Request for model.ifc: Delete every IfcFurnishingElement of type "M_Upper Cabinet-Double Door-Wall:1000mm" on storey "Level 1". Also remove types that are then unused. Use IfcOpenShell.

First a look at what the model holds.

```python
import ifcopenshell
import ifcopenshell.util.element

model = ifcopenshell.open("model.ifc")
print(model.schema)
storey = next(s for s in model.by_type("IfcBuildingStorey") if s.Name == "Level 1")
furniture = [e for e in ifcopenshell.util.element.get_decomposition(storey) if e.is_a("IfcFurnishingElement")]
seen = {}
for e in furniture:
    element_type = ifcopenshell.util.element.get_type(e)
    name = element_type.Name if element_type not in (None, e) else None
    seen[name] = seen.get(name, 0) + 1
for name, count in sorted(seen.items(), key=str):
    print(count, "x", name)
```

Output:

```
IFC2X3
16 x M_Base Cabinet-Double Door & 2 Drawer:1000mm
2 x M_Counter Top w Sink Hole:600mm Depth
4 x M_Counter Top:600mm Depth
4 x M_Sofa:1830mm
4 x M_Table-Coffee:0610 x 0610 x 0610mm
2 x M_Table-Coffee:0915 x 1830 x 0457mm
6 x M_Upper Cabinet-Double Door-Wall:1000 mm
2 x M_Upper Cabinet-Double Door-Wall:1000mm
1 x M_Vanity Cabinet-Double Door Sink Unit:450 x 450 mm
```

```python
import ifcopenshell
import ifcopenshell.api.root
import ifcopenshell.util.element

model = ifcopenshell.open("model.ifc")

storey = next(s for s in model.by_type("IfcBuildingStorey") if s.Name == "Level 1")
furniture = [e for e in ifcopenshell.util.element.get_decomposition(storey) if e.is_a("IfcFurnishingElement")]
targets = [e for e in furniture if (t := ifcopenshell.util.element.get_type(e)) not in (None, e) and t.Name == "M_Upper Cabinet-Double Door-Wall:1000mm"]
types = {ifcopenshell.util.element.get_type(e) for e in targets} - {None, *targets}

for e in targets:
    ifcopenshell.api.root.remove_product(model, product=e)
print(len(targets), "removed")

unused = [t for t in types if not ifcopenshell.util.element.get_types(t)]
for t in unused:
    ifcopenshell.api.root.remove_product(model, product=t)
print(len(unused), "unused types removed")

model.write("model_updated.ifc")
```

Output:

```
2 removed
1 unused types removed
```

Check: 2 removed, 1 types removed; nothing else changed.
